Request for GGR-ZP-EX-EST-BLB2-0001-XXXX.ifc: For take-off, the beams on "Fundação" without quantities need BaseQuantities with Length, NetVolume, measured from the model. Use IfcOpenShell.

First a look at what the model holds.

```python
import ifcopenshell
import ifcopenshell.util.element
import ifcopenshell.util.unit

model = ifcopenshell.open("GGR-ZP-EX-EST-BLB2-0001-XXXX.ifc")
print(model.schema)
for unit_type in ("LENGTHUNIT", "AREAUNIT", "VOLUMEUNIT"):
    print(unit_type, ifcopenshell.util.unit.calculate_unit_scale(model, unit_type))
storey = next(s for s in model.by_type("IfcBuildingStorey") if s.Name == "Fundação")
beams = [e for e in ifcopenshell.util.element.get_decomposition(storey) if e.is_a("IfcBeam")]
for e in sorted(beams, key=lambda e: e.id()):
    print(e.id(), e.is_a(), e.Name, list(ifcopenshell.util.element.get_psets(e, qtos_only=True)), sep=" | ")
```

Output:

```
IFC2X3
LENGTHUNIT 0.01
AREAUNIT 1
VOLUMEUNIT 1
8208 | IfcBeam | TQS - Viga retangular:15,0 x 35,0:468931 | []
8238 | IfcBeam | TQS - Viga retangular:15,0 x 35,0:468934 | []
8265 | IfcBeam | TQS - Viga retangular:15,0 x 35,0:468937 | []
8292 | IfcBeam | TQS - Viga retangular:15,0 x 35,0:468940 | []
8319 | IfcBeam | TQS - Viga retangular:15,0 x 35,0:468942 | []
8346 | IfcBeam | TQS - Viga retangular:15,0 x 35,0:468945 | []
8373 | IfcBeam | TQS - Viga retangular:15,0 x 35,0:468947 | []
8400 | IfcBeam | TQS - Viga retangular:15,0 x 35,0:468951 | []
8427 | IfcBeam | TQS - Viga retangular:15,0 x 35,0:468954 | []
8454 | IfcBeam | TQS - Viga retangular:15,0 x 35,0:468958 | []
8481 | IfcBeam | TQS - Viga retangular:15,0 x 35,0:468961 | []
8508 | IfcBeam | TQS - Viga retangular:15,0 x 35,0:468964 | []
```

```python
import ifcopenshell
import ifcopenshell.api.pset
import ifcopenshell.geom
import ifcopenshell.util.element
import ifcopenshell.util.shape
import ifcopenshell.util.unit

model = ifcopenshell.open("GGR-ZP-EX-EST-BLB2-0001-XXXX.ifc")
unit_scale = ifcopenshell.util.unit.calculate_unit_scale(model)
volume_scale = ifcopenshell.util.unit.calculate_unit_scale(model, "VOLUMEUNIT")
settings = ifcopenshell.geom.settings()

storey = next(s for s in model.by_type("IfcBuildingStorey") if s.Name == "Fundação")
beams = [e for e in ifcopenshell.util.element.get_decomposition(storey) if e.is_a("IfcBeam")]

for e in sorted(beams, key=lambda e: e.id()):
    if ifcopenshell.util.element.get_psets(e, qtos_only=True, should_inherit=False):
        continue
    # Geometry comes back in metres, in the element's own axes.
    shape = ifcopenshell.geom.create_shape(settings, e)
    values = {
        "Length": ifcopenshell.util.shape.get_max_xyz(shape.geometry) / unit_scale,
        "NetVolume": ifcopenshell.util.shape.get_volume(shape.geometry) / volume_scale,
    }
    qto = ifcopenshell.api.pset.add_qto(model, product=e, name="BaseQuantities")
    ifcopenshell.api.pset.edit_qto(model, qto=qto, properties=values)
    print(e.id(), {k: round(v, 3) for k, v in values.items()})

model.write("GGR-ZP-EX-EST-BLB2-0001-XXXX_updated.ifc")
```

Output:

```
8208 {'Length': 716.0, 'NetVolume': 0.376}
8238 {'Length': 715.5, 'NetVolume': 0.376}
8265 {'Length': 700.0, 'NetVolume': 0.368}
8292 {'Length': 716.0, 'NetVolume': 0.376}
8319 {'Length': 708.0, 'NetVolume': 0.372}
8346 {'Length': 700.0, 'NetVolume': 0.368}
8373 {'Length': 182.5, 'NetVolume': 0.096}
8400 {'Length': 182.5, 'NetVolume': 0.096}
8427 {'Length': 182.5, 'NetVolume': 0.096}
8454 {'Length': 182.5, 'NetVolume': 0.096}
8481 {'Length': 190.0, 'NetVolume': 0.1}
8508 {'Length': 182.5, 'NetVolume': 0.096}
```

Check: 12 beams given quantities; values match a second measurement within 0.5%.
